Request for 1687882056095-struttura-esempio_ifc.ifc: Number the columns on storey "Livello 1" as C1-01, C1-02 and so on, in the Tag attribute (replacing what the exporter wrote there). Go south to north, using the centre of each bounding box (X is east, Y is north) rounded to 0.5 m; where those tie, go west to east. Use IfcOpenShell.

First a look at what the model holds.

```python
import ifcopenshell
import ifcopenshell.util.element
import ifcopenshell.util.placement

model = ifcopenshell.open("1687882056095-struttura-esempio_ifc.ifc")
print(model.schema)
storey = next(s for s in model.by_type("IfcBuildingStorey") if s.Name == "Livello 1")
columns = [e for e in ifcopenshell.util.element.get_decomposition(storey) if e.is_a("IfcColumn")]
for e in sorted(columns, key=lambda e: e.id()):
    origin = ifcopenshell.util.placement.get_local_placement(e.ObjectPlacement)[:3, 3]
    print(e.id(), e.Tag, e.Name, origin.round(2) + 0.0, sep=" | ")
```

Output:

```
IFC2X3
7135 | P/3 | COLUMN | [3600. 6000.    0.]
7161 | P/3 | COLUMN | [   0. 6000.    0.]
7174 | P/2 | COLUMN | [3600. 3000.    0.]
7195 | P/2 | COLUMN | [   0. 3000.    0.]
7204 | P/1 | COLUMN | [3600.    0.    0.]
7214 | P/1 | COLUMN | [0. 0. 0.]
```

```python
import ifcopenshell
import ifcopenshell.geom
import ifcopenshell.util.element
import ifcopenshell.util.shape

model = ifcopenshell.open("1687882056095-struttura-esempio_ifc.ifc")
settings = ifcopenshell.geom.settings()
settings.set("use-world-coords", True)


def centre(element):
    shape = ifcopenshell.geom.create_shape(settings, element)
    return ifcopenshell.util.shape.get_bbox_centroid(shape.geometry)


storey = next(s for s in model.by_type("IfcBuildingStorey") if s.Name == "Livello 1")
columns = [e for e in ifcopenshell.util.element.get_decomposition(storey) if e.is_a("IfcColumn")]

# Insertion points can sit at a corner or the storey origin, so sort by the geometry (in metres).
centres = {e: centre(e) for e in columns}
columns.sort(key=lambda e: (round(centres[e][1] / 0.5), centres[e][0]))

for i, e in enumerate(columns, start=1):
    number = f"C1-{i:02d}"
    e.Tag = number
    print(e.id(), number)

model.write("1687882056095-struttura-esempio_ifc_v2.ifc")
```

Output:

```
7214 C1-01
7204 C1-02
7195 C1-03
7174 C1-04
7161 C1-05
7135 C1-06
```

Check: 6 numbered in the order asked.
